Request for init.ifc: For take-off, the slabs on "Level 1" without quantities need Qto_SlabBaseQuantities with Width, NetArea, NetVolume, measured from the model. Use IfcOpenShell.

First a look at what the model holds.

```python
import ifcopenshell
import ifcopenshell.util.element
import ifcopenshell.util.unit

model = ifcopenshell.open("init.ifc")
print(model.schema)
for unit_type in ("LENGTHUNIT", "AREAUNIT", "VOLUMEUNIT"):
    print(unit_type, ifcopenshell.util.unit.calculate_unit_scale(model, unit_type))
storey = next(s for s in model.by_type("IfcBuildingStorey") if s.Name == "Level 1")
slabs = [e for e in ifcopenshell.util.element.get_decomposition(storey) if e.is_a("IfcSlab")]
for e in sorted(slabs, key=lambda e: e.id()):
    print(e.id(), e.is_a(), e.Name, list(ifcopenshell.util.element.get_psets(e, qtos_only=True)), sep=" | ")
```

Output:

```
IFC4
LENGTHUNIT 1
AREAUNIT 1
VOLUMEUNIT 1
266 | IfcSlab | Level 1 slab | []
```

```python
import ifcopenshell
import ifcopenshell.api.pset
import ifcopenshell.geom
import ifcopenshell.util.element
import ifcopenshell.util.shape
import ifcopenshell.util.unit

model = ifcopenshell.open("init.ifc")
unit_scale = ifcopenshell.util.unit.calculate_unit_scale(model)
area_scale = ifcopenshell.util.unit.calculate_unit_scale(model, "AREAUNIT")
volume_scale = ifcopenshell.util.unit.calculate_unit_scale(model, "VOLUMEUNIT")
settings = ifcopenshell.geom.settings()

storey = next(s for s in model.by_type("IfcBuildingStorey") if s.Name == "Level 1")
slabs = [e for e in ifcopenshell.util.element.get_decomposition(storey) if e.is_a("IfcSlab")]

for e in sorted(slabs, key=lambda e: e.id()):
    if ifcopenshell.util.element.get_psets(e, qtos_only=True, should_inherit=False):
        continue
    # Geometry comes back in metres, in the element's own axes.
    shape = ifcopenshell.geom.create_shape(settings, e)
    values = {
        "Width": ifcopenshell.util.shape.get_z(shape.geometry) / unit_scale,
        "NetArea": ifcopenshell.util.shape.get_footprint_area(shape.geometry) / area_scale,
        "NetVolume": ifcopenshell.util.shape.get_volume(shape.geometry) / volume_scale,
    }
    qto = ifcopenshell.api.pset.add_qto(model, product=e, name="Qto_SlabBaseQuantities")
    ifcopenshell.api.pset.edit_qto(model, qto=qto, properties=values)
    print(e.id(), {k: round(v, 3) for k, v in values.items()})

model.write("init_v2.ifc")
```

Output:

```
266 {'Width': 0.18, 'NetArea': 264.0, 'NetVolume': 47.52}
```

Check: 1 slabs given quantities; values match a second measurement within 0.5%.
